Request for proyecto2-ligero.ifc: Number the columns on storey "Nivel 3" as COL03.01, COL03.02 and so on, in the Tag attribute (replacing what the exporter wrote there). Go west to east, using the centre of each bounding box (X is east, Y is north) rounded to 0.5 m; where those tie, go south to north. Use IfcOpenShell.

First a look at what the model holds.

```python
import ifcopenshell
import ifcopenshell.util.element
import ifcopenshell.util.placement

model = ifcopenshell.open("proyecto2-ligero.ifc")
print(model.schema)
storey = next(s for s in model.by_type("IfcBuildingStorey") if s.Name == "Nivel 3")
columns = [e for e in ifcopenshell.util.element.get_decomposition(storey) if e.is_a("IfcColumn")]
for e in sorted(columns, key=lambda e: e.id()):
    origin = ifcopenshell.util.placement.get_local_placement(e.ObjectPlacement)[:3, 3]
    print(e.id(), e.Tag, e.Name, origin.round(2) + 0.0, sep=" | ")
```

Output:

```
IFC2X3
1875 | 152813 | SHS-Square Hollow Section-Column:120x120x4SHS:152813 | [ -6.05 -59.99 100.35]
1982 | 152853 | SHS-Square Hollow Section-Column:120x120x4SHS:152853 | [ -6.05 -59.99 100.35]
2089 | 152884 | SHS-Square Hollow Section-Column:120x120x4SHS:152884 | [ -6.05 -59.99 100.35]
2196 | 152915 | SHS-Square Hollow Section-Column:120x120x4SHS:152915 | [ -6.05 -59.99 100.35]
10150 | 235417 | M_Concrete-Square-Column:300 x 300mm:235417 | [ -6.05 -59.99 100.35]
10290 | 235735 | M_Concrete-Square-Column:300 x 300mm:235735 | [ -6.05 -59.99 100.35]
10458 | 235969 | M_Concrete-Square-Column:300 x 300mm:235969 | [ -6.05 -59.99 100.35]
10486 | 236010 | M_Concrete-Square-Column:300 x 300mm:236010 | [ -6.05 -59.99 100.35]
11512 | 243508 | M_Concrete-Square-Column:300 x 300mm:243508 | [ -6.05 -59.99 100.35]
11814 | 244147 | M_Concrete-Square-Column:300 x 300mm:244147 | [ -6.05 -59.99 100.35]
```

```python
import ifcopenshell
import ifcopenshell.geom
import ifcopenshell.util.element
import ifcopenshell.util.shape

model = ifcopenshell.open("proyecto2-ligero.ifc")
settings = ifcopenshell.geom.settings()
settings.set("use-world-coords", True)


def centre(element):
    shape = ifcopenshell.geom.create_shape(settings, element)
    return ifcopenshell.util.shape.get_bbox_centroid(shape.geometry)


storey = next(s for s in model.by_type("IfcBuildingStorey") if s.Name == "Nivel 3")
columns = [e for e in ifcopenshell.util.element.get_decomposition(storey) if e.is_a("IfcColumn")]

# Insertion points can sit at a corner or the storey origin, so sort by the geometry (in metres).
centres = {e: centre(e) for e in columns}
columns.sort(key=lambda e: (round(centres[e][0] / 0.5), centres[e][1]))

for i, e in enumerate(columns, start=1):
    number = f"COL03.{i:02d}"
    e.Tag = number
    print(e.id(), number)

model.write("proyecto2-ligero_v2.ifc")
```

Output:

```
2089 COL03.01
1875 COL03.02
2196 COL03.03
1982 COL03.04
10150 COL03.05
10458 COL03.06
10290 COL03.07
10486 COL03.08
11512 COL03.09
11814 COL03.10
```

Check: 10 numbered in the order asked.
